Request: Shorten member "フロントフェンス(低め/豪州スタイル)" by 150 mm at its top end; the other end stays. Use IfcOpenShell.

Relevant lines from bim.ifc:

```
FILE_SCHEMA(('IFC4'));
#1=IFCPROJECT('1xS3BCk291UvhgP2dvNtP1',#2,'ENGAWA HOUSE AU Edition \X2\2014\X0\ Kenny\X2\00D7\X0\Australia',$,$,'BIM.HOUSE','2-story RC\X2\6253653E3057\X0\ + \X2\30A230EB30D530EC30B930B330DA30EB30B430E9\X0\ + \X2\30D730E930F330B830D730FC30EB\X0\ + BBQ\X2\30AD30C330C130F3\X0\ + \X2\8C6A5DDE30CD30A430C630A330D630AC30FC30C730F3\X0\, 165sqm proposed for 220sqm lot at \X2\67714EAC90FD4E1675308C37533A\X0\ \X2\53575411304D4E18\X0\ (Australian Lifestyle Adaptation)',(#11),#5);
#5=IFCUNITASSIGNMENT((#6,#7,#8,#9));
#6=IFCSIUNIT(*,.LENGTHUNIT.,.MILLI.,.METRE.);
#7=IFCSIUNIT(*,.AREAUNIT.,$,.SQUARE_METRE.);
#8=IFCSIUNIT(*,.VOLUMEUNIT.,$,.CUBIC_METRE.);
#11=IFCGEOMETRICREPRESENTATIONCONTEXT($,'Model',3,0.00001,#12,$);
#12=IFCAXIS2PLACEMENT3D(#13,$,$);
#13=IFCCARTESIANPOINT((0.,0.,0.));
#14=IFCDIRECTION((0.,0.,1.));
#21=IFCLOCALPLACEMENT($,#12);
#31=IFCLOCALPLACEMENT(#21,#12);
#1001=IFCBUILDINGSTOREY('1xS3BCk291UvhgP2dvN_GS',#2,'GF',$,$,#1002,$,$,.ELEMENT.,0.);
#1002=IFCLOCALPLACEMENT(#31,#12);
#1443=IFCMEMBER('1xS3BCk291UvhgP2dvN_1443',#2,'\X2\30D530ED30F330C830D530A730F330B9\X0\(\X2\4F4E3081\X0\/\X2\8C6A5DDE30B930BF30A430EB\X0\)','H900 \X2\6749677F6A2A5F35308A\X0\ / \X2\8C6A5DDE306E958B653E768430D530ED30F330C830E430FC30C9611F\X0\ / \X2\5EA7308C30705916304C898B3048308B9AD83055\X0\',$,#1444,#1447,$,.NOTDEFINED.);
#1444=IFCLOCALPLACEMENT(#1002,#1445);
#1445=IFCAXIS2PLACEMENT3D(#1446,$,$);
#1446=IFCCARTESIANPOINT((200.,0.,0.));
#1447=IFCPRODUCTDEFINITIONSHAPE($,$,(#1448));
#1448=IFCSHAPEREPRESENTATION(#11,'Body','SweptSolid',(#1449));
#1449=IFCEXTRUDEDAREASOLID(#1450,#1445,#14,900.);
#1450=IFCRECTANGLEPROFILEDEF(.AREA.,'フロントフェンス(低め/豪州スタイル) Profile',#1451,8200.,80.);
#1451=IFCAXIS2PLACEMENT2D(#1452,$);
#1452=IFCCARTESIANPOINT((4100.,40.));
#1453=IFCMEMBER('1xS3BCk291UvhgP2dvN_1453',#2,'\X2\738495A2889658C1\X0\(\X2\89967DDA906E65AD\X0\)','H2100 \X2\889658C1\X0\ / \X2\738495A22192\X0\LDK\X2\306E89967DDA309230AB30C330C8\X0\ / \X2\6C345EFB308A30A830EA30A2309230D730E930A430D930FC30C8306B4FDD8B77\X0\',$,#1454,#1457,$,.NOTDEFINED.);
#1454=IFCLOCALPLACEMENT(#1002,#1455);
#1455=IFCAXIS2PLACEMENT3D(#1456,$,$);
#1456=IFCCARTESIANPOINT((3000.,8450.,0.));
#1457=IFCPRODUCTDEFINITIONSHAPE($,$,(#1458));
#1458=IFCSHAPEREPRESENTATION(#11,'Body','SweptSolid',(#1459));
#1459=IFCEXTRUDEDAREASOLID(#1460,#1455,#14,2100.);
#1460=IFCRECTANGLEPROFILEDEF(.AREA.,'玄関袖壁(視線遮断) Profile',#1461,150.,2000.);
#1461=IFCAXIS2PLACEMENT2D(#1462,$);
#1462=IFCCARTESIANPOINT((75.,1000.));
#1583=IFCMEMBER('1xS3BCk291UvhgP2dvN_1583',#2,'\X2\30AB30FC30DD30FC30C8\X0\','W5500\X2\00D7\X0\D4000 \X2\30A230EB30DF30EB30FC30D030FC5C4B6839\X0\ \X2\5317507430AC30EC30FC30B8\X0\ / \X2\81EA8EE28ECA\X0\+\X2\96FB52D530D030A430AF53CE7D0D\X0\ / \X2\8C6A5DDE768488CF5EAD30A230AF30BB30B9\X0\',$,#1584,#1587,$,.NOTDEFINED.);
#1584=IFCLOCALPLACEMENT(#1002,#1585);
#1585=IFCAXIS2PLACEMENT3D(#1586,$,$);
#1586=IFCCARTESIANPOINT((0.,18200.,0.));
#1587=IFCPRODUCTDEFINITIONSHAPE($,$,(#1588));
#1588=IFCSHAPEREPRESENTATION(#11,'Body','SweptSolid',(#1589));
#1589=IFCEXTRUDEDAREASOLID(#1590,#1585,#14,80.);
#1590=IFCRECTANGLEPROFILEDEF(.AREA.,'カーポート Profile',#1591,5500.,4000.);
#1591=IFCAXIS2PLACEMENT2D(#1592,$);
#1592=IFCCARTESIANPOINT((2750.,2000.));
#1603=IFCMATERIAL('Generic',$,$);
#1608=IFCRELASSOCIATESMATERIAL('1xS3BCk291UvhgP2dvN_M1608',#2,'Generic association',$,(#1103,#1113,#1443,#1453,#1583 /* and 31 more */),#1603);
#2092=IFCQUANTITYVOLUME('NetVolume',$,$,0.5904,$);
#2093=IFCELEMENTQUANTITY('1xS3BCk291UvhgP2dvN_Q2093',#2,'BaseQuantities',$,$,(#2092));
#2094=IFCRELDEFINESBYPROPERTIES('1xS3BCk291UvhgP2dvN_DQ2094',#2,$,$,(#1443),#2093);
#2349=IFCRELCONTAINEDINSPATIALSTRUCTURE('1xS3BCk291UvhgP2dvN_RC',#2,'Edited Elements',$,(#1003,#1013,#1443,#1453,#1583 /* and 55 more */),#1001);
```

```python
import ifcopenshell
import ifcopenshell.api.pset
import ifcopenshell.util.element
import ifcopenshell.util.unit

model = ifcopenshell.open("bim.ifc")
unit_scale = ifcopenshell.util.unit.calculate_unit_scale(model)

member = model.by_guid("1xS3BCk291UvhgP2dvN_1443")
change = -0.15 / unit_scale

# The extrusion runs towards the end named, so only its depth changes.
body = next(r for r in member.Representation.Representations if r.RepresentationIdentifier == "Body")
solid = body.Items[0]
old_length = solid.Depth
solid.Depth += change

# Update the stored length and volume.
qto = model.by_id(ifcopenshell.util.element.get_pset(member, "BaseQuantities", should_inherit=False)["id"])
ifcopenshell.api.pset.edit_qto(model, qto=qto, properties={
    "NetVolume": ifcopenshell.util.element.get_pset(member, "BaseQuantities", "NetVolume") * solid.Depth / old_length,
})

print(f"length {old_length:g} -> {solid.Depth:g}")

model.write("bim_v2.ifc")
```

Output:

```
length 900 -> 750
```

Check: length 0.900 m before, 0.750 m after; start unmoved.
